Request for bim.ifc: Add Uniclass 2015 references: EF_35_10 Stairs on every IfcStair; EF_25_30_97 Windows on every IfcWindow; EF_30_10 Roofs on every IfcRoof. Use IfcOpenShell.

First a look at what the model holds.

```python
import ifcopenshell

model = ifcopenshell.open("bim.ifc")
print(model.schema)
print("classifications:", [c.Name for c in model.by_type("IfcClassification")])
for ifc_class in ("IfcDoor", "IfcRoof", "IfcStair", "IfcWall", "IfcWindow"):
    print(ifc_class, len(model.by_type(ifc_class)))
```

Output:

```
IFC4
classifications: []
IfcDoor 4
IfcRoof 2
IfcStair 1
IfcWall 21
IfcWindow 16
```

```python
import ifcopenshell
import ifcopenshell.api.classification

model = ifcopenshell.open("bim.ifc")

system = ifcopenshell.api.classification.add_classification(model, classification="Uniclass 2015")

codes = {
    "IfcStair": ("EF_35_10", "Stairs"),
    "IfcWindow": ("EF_25_30_97", "Windows"),
    "IfcRoof": ("EF_30_10", "Roofs"),
}
for ifc_class, (code, name) in codes.items():
    products = model.by_type(ifc_class)
    ifcopenshell.api.classification.add_reference(
        model, products=products, classification=system, identification=code, name=name
    )
    print(code, len(products))

model.write("bim_edited.ifc")
```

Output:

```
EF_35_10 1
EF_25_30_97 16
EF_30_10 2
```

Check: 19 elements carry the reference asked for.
